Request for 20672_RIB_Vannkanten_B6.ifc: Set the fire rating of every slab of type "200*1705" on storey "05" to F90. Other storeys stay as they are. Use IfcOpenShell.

First a look at what the model holds.

```python
import ifcopenshell
import ifcopenshell.util.element

model = ifcopenshell.open("20672_RIB_Vannkanten_B6.ifc")
print(model.schema)
storey = next(s for s in model.by_type("IfcBuildingStorey") if s.Name == "05")
slabs = [e for e in ifcopenshell.util.element.get_decomposition(storey) if e.is_a("IfcSlab")]
seen = {}
for e in slabs:
    element_type = ifcopenshell.util.element.get_type(e)
    key = (element_type.Name if element_type != e and element_type else None, ifcopenshell.util.element.get_pset(e, "Pset_SlabCommon", "FireRating"))
    seen[key] = seen.get(key, 0) + 1
for (name, value), count in sorted(seen.items(), key=str):
    print(count, "x", name, "|", value)
```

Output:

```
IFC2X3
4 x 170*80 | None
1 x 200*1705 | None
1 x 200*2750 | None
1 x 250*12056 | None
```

```python
import ifcopenshell
import ifcopenshell.api.pset
import ifcopenshell.util.element

model = ifcopenshell.open("20672_RIB_Vannkanten_B6.ifc")

storey = next(s for s in model.by_type("IfcBuildingStorey") if s.Name == "05")
slabs = [e for e in ifcopenshell.util.element.get_decomposition(storey) if e.is_a("IfcSlab")]

count = 0
for e in slabs:
    element_type = ifcopenshell.util.element.get_type(e)
    if element_type in (None, e) or element_type.Name != "200*1705":
        continue
    # add_pset returns the element's existing set when there is one.
    pset = ifcopenshell.api.pset.add_pset(model, product=e, name="Pset_SlabCommon")
    ifcopenshell.api.pset.edit_pset(model, pset=pset, properties={"FireRating": "F90"})
    count += 1

print(count, "slabs updated")

model.write("20672_RIB_Vannkanten_B6-out.ifc")
```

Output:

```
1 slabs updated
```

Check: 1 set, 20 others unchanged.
